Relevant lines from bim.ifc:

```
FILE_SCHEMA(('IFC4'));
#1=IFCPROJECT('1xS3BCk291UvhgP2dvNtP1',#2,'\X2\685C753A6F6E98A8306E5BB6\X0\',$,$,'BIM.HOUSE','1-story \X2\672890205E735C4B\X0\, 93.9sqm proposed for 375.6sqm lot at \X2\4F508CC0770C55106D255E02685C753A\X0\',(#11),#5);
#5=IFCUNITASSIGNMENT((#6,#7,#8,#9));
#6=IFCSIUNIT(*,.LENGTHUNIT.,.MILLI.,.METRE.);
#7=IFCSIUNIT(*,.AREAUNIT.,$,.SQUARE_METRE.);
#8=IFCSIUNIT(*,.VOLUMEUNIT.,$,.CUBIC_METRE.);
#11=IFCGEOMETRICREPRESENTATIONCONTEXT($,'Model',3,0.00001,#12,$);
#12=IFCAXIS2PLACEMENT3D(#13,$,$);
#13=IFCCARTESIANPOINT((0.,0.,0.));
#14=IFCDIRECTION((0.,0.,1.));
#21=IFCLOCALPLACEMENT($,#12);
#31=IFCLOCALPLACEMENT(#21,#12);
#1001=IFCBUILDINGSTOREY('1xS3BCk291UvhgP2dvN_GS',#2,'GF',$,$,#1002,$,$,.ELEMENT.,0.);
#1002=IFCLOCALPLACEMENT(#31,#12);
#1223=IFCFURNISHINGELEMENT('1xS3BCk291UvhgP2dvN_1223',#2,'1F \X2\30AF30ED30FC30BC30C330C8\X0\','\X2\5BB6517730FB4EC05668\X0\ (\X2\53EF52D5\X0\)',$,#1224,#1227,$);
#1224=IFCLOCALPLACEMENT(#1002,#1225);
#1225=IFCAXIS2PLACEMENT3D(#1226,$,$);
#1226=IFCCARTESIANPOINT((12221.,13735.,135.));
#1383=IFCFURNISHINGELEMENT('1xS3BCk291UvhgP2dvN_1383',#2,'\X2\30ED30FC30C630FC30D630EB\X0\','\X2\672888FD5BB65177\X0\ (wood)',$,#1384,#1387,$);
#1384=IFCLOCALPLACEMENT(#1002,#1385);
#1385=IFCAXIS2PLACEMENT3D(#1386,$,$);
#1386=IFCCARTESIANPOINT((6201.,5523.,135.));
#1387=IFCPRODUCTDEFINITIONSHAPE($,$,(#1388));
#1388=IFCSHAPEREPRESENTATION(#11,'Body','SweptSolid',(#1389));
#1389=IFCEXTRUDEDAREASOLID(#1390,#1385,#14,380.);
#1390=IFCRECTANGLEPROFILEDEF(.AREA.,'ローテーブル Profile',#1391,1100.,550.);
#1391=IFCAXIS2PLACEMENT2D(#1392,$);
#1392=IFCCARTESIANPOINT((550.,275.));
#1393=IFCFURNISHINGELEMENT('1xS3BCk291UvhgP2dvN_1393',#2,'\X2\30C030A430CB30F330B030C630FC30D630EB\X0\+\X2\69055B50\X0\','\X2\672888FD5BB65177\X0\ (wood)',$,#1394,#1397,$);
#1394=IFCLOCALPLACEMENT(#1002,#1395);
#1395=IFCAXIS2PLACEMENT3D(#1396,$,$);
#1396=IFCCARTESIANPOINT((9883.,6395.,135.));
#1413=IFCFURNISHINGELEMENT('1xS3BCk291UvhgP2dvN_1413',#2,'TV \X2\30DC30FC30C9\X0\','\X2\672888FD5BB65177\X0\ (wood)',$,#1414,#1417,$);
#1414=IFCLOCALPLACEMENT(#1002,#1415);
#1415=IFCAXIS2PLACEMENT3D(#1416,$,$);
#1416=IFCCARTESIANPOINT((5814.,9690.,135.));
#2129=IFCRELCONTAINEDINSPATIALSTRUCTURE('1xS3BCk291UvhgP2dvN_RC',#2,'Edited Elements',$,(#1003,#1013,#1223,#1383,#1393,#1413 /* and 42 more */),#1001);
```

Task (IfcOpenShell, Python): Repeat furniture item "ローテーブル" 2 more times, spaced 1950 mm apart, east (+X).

```python
import numpy as np
import ifcopenshell
import ifcopenshell.api.geometry
import ifcopenshell.api.root
import ifcopenshell.util.element
import ifcopenshell.util.placement

model = ifcopenshell.open("bim.ifc")


def reuse_history(source, copy):
    """copy_class also copies each property set's owner history, people and application; keep the originals."""
    for rel in copy.IsDefinedBy:
        if rel.is_a("IfcRelDefinesByProperties") and (history := rel.RelatingPropertyDefinition.OwnerHistory):
            rel.RelatingPropertyDefinition.OwnerHistory = source.OwnerHistory
            ifcopenshell.util.element.remove_deep2(model, history)


source = model.by_guid("1xS3BCk291UvhgP2dvN_1383")
base = ifcopenshell.util.placement.get_local_placement(source.ObjectPlacement)
step = np.array([1.0, 0.0, 0.0]) * 1950.0

for i in range(1, 3):
    copy = ifcopenshell.api.root.copy_class(model, product=source)
    copy.Representation = ifcopenshell.util.element.copy_deep(
        model, source.Representation, exclude=["IfcGeometricRepresentationContext", "IfcRepresentationMap"]
    )
    reuse_history(source, copy)
    matrix = base.copy()
    matrix[:3, 3] += i * step
    print("added at", matrix[:3, 3].round(3) + 0.0)
    ifcopenshell.api.geometry.edit_object_placement(model, product=copy, matrix=matrix, is_si=False)

model.write("bim_edited.ifc")
```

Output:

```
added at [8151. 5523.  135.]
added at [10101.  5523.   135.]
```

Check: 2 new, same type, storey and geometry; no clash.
